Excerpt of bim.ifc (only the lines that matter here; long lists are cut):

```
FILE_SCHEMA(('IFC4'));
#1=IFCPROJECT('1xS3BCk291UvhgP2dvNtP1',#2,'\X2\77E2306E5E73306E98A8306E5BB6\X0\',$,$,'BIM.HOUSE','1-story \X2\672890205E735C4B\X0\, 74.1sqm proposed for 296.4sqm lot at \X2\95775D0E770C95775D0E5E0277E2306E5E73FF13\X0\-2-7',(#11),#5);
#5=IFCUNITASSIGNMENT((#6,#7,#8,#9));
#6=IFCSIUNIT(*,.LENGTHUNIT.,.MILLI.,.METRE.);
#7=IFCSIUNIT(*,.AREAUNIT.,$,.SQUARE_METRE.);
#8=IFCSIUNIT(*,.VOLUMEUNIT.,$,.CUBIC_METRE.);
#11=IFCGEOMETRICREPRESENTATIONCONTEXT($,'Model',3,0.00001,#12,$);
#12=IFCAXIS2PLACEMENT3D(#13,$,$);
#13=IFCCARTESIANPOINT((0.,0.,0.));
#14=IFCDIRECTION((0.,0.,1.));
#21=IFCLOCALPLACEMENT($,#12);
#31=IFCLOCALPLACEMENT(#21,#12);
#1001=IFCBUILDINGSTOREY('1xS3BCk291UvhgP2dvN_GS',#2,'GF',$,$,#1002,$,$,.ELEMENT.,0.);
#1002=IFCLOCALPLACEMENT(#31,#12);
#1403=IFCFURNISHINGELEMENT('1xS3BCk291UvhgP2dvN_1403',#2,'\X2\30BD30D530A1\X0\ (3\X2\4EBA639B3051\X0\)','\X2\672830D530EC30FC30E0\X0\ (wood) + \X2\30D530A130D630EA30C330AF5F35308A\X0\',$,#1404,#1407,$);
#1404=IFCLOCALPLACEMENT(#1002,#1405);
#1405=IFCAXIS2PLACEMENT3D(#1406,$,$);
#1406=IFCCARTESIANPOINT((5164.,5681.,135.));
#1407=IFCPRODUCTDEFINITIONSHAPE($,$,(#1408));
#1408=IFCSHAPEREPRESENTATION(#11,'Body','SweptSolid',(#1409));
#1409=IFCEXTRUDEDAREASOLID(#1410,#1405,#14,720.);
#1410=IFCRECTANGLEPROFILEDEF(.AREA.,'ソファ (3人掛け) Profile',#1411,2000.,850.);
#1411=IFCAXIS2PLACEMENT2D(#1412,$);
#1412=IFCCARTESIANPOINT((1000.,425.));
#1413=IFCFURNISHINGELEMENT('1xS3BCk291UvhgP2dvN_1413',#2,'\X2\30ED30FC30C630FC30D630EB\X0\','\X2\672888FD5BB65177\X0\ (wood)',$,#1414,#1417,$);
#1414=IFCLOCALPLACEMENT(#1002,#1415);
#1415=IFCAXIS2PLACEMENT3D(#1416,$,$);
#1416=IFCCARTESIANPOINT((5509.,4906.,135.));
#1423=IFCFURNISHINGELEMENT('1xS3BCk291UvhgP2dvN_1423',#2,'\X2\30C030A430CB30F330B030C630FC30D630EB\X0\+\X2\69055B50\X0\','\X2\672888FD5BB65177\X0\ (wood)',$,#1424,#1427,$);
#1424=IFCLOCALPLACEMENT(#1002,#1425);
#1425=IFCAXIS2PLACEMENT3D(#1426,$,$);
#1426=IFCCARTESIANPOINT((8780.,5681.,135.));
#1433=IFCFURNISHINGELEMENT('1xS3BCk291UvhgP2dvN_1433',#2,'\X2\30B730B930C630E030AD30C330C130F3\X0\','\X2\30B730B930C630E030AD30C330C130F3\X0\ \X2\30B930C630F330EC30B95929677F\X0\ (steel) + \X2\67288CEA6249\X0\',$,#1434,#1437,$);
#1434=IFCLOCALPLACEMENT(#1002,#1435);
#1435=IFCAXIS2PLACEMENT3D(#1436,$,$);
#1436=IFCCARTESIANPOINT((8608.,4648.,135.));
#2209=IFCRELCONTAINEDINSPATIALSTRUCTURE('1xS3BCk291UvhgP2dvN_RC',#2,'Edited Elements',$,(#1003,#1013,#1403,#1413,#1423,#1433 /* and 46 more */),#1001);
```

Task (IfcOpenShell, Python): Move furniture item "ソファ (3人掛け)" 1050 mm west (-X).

```python
import ifcopenshell
import ifcopenshell.api.geometry
import ifcopenshell.util.placement

model = ifcopenshell.open("bim.ifc")

item = model.by_guid("1xS3BCk291UvhgP2dvN_1403")
matrix = ifcopenshell.util.placement.get_local_placement(item.ObjectPlacement)
matrix[0, 3] -= 1050.0
ifcopenshell.api.geometry.edit_object_placement(model, product=item, matrix=matrix, is_si=False)

print(ifcopenshell.util.placement.get_local_placement(item.ObjectPlacement).round(3) + 0.0)

model.write("bim_edited.ifc")
```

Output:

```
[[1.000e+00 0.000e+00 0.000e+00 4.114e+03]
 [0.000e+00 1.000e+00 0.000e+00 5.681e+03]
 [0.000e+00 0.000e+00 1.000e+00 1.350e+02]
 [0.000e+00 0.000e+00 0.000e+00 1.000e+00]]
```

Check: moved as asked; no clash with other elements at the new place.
